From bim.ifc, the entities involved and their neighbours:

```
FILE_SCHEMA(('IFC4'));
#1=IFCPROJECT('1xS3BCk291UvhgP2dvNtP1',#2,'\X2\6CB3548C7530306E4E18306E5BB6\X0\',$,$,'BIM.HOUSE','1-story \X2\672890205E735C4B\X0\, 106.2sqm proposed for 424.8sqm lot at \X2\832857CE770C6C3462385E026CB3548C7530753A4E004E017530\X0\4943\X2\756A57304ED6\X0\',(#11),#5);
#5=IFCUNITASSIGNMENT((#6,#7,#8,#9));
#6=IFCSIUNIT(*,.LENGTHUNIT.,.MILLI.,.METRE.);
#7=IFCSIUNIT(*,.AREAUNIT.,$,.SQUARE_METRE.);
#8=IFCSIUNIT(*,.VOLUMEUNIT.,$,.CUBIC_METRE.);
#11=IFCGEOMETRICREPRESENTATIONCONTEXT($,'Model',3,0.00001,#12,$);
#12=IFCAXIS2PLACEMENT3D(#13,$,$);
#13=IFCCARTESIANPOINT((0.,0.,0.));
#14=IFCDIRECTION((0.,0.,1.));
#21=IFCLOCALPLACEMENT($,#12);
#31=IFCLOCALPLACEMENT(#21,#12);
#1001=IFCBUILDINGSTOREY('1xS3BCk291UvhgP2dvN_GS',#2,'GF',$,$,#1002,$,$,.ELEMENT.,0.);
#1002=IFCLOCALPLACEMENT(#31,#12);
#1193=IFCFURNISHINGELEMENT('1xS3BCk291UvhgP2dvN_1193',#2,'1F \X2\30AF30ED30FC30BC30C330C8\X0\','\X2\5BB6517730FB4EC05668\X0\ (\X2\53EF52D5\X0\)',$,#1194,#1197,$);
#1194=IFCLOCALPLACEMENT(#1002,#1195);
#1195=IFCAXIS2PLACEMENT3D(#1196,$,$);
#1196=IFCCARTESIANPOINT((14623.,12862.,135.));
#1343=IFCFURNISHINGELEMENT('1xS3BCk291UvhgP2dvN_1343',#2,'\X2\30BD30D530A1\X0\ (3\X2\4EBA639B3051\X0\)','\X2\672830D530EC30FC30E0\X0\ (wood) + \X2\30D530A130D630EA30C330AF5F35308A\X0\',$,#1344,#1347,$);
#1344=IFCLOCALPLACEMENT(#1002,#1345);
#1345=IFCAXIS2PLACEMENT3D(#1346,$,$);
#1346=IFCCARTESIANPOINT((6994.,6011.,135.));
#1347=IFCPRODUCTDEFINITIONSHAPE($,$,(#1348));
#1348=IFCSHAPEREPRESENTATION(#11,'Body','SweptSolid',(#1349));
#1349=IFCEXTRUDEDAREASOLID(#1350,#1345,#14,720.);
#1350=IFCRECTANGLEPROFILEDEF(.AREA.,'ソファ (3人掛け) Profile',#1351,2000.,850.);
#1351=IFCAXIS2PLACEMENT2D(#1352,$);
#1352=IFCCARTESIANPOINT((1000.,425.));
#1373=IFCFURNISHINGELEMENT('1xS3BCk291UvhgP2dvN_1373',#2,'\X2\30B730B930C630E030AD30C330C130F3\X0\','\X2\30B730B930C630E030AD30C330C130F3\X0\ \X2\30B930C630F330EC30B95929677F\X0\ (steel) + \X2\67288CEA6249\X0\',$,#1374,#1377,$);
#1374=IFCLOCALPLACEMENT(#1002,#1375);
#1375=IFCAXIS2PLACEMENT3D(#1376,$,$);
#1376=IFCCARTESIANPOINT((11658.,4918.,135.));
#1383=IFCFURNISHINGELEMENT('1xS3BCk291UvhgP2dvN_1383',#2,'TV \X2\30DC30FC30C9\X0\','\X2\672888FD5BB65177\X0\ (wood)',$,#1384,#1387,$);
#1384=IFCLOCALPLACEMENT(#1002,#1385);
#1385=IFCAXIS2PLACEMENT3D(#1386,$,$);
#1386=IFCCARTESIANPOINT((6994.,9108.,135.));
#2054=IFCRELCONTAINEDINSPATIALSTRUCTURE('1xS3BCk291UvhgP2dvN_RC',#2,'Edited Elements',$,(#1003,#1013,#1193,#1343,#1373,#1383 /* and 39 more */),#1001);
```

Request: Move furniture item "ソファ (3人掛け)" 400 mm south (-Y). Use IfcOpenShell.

```python
import ifcopenshell
import ifcopenshell.api.geometry
import ifcopenshell.util.placement

model = ifcopenshell.open("bim.ifc")

item = model.by_guid("1xS3BCk291UvhgP2dvN_1343")
matrix = ifcopenshell.util.placement.get_local_placement(item.ObjectPlacement)
matrix[1, 3] -= 400.0
ifcopenshell.api.geometry.edit_object_placement(model, product=item, matrix=matrix, is_si=False)

print(ifcopenshell.util.placement.get_local_placement(item.ObjectPlacement).round(3) + 0.0)

model.write("bim_edited.ifc")
```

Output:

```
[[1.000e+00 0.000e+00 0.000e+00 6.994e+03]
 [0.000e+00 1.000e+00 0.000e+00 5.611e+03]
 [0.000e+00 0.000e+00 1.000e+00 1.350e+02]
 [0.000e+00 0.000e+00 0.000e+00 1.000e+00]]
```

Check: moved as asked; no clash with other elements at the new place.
